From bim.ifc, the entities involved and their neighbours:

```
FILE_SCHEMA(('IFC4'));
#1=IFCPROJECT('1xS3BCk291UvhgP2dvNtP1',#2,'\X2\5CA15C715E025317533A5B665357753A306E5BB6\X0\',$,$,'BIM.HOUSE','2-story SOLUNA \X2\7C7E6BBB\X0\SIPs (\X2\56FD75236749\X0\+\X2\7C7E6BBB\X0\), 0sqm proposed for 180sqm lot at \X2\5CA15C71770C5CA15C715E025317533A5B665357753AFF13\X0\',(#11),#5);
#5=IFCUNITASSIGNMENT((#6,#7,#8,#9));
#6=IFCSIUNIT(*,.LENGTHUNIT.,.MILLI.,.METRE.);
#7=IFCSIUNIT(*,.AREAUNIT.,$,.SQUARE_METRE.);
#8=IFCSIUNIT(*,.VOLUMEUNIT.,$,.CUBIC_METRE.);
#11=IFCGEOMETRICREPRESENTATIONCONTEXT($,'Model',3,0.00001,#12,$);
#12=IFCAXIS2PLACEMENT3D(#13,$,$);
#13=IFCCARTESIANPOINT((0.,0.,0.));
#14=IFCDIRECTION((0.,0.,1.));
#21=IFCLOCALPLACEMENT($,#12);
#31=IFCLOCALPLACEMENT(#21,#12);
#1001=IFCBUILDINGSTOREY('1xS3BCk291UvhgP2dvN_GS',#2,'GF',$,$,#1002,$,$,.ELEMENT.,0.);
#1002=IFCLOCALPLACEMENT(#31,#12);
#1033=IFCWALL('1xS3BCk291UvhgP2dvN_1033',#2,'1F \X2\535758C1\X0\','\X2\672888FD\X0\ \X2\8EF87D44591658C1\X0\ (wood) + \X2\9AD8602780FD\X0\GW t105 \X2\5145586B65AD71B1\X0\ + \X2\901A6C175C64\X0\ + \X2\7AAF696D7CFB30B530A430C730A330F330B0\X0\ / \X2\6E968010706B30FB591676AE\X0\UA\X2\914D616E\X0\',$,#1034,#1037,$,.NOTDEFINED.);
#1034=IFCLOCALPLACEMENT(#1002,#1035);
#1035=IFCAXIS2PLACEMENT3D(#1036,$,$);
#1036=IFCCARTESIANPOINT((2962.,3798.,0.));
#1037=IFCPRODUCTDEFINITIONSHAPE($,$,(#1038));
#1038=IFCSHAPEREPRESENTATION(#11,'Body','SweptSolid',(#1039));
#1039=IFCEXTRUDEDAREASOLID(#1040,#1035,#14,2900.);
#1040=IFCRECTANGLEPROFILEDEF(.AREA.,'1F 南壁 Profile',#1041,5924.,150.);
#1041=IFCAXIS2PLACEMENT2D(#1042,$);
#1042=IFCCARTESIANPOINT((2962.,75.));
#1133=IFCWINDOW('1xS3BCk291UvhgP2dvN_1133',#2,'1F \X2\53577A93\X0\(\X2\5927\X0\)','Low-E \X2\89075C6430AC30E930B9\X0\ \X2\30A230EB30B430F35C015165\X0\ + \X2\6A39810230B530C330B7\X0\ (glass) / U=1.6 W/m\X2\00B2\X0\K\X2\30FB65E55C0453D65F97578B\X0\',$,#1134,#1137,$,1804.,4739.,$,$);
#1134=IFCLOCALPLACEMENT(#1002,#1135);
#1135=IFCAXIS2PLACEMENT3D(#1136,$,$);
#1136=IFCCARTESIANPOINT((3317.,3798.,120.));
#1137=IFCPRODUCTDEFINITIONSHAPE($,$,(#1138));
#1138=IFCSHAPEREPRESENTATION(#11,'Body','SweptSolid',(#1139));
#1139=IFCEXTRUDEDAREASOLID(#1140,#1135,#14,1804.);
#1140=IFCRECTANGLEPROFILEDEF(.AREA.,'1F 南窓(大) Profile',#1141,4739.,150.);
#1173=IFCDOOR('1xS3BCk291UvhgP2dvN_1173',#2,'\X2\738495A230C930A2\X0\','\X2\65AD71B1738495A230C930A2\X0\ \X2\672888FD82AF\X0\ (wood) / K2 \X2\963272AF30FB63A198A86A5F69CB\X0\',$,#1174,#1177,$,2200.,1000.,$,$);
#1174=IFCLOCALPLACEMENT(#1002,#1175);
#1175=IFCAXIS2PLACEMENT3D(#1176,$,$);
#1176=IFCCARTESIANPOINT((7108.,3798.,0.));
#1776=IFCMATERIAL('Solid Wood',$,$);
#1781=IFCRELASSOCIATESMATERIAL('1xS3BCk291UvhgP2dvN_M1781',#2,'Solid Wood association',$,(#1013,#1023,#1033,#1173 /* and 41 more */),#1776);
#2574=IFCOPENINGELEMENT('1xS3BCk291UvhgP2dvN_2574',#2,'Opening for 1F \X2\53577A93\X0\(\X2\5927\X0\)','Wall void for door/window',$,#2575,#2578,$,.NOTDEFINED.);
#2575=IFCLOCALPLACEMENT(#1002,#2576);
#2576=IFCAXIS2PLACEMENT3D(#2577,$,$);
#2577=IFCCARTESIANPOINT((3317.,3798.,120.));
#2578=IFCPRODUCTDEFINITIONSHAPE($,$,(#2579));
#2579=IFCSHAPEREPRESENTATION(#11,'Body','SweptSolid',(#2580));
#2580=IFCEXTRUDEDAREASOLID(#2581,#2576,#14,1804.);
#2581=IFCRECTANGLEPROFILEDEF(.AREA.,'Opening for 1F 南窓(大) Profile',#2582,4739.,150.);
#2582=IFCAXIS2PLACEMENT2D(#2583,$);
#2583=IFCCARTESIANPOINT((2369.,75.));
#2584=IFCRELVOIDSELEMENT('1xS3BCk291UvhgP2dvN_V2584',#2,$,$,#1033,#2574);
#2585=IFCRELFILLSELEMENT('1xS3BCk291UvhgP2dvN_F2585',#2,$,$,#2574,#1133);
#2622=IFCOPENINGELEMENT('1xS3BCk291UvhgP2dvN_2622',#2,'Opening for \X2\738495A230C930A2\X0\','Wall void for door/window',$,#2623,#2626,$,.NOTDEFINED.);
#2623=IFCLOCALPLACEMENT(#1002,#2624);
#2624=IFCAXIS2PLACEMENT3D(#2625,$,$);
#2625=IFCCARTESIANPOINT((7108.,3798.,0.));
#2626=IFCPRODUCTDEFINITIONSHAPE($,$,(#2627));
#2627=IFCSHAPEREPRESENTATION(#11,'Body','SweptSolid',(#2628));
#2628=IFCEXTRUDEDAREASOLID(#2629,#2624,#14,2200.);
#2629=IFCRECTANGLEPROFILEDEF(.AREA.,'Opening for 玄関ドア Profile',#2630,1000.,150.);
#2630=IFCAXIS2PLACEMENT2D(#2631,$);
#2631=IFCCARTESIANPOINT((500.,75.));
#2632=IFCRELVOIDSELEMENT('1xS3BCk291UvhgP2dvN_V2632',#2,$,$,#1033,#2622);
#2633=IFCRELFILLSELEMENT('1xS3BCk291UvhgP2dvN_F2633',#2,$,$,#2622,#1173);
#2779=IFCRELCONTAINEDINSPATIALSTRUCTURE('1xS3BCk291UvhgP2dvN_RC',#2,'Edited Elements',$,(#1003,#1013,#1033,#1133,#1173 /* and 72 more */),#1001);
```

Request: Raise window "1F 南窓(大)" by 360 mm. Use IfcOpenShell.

```python
import numpy as np
import ifcopenshell
import ifcopenshell.api.geometry
import ifcopenshell.util.placement
import ifcopenshell.util.unit

model = ifcopenshell.open("bim.ifc")
unit_scale = ifcopenshell.util.unit.calculate_unit_scale(model)

window = model.by_guid("1xS3BCk291UvhgP2dvN_1133")
opening = window.FillsVoids[0].RelatingOpeningElement
dz = 0.36 / unit_scale

shift = np.array([0.0, 0.0, dz])
# The window is not placed relative to its opening, so move both.
for product in (opening, window):
    matrix = ifcopenshell.util.placement.get_local_placement(product.ObjectPlacement)
    matrix[:3, 3] += shift
    ifcopenshell.api.geometry.edit_object_placement(model, product=product, matrix=matrix, is_si=False)

print(f"moved by {dz * unit_scale:+.3f} m")

model.write("bim_updated.ifc")
```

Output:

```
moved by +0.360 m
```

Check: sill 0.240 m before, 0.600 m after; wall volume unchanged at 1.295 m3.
